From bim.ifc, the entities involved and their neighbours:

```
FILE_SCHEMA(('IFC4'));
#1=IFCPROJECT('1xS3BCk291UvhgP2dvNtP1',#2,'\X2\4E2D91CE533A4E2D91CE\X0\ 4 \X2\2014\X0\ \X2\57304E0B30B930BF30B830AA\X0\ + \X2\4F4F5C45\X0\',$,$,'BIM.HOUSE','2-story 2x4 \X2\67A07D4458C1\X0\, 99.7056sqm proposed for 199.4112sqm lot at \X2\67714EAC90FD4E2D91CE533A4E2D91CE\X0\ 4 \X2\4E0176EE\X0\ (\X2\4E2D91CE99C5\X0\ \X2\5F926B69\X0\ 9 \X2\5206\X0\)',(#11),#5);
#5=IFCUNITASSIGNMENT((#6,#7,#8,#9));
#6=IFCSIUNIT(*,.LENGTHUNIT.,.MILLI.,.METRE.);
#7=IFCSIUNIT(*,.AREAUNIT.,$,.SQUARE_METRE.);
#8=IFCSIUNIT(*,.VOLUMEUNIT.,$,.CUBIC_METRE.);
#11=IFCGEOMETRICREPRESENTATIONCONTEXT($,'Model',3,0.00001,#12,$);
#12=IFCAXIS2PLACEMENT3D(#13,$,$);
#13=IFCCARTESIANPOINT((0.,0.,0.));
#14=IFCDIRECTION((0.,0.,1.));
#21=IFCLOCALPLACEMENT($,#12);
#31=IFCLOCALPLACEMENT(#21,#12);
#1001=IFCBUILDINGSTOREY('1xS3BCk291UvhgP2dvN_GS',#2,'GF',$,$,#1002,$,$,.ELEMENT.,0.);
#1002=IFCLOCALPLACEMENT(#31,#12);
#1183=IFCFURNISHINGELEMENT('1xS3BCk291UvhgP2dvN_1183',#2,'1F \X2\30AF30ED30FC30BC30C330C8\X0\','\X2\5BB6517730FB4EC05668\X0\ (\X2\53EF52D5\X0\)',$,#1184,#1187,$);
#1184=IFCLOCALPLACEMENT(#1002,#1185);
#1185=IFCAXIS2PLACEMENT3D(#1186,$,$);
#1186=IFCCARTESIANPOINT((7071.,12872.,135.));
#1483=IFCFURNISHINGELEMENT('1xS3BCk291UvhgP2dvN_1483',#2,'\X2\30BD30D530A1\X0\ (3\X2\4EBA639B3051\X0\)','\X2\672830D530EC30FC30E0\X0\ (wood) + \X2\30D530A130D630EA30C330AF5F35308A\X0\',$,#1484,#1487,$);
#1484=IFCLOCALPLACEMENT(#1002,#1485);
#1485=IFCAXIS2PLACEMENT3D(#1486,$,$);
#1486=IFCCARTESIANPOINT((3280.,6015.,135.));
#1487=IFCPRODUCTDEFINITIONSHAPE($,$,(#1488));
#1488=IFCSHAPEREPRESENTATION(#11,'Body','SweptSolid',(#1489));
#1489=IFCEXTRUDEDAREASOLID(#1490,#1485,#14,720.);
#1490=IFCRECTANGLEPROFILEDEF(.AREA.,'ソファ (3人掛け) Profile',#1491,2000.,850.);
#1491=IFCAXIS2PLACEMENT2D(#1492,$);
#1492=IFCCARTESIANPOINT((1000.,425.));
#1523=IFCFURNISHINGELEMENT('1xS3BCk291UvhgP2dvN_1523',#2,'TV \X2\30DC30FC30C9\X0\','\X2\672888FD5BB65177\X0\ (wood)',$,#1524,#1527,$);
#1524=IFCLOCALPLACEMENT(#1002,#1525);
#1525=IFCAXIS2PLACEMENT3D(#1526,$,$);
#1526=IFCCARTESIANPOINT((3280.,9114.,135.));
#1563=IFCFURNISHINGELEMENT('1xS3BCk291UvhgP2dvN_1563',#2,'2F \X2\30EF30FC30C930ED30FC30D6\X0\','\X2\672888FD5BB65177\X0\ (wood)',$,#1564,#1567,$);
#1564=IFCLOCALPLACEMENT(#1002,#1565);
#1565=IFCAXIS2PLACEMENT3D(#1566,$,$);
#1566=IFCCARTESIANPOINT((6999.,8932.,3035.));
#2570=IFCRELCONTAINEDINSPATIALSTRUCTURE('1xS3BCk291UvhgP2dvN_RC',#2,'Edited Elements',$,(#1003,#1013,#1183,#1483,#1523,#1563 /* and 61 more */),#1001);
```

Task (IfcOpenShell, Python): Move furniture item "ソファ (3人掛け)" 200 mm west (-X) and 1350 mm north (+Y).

```python
import ifcopenshell
import ifcopenshell.api.geometry
import ifcopenshell.util.placement
import ifcopenshell.util.unit

model = ifcopenshell.open("bim.ifc")
unit_scale = ifcopenshell.util.unit.calculate_unit_scale(model)

item = model.by_guid("1xS3BCk291UvhgP2dvN_1483")
matrix = ifcopenshell.util.placement.get_local_placement(item.ObjectPlacement)
matrix[0, 3] -= 0.2 / unit_scale
matrix[1, 3] += 1.35 / unit_scale
ifcopenshell.api.geometry.edit_object_placement(model, product=item, matrix=matrix, is_si=False)

print(ifcopenshell.util.placement.get_local_placement(item.ObjectPlacement).round(3) + 0.0)

model.write("bim_updated.ifc")
```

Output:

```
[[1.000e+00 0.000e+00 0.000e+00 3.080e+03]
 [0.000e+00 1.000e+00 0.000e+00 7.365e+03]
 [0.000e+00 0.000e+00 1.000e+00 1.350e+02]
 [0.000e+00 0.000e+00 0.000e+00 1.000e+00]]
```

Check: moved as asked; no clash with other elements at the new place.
